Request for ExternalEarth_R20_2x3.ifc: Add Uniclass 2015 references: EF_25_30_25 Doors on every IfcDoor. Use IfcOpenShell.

First a look at what the model holds.

```python
import ifcopenshell

model = ifcopenshell.open("ExternalEarth_R20_2x3.ifc")
print(model.schema)
print("classifications:", [c.Name for c in model.by_type("IfcClassification")])
for ifc_class in ("IfcDoor", "IfcRoof", "IfcStair", "IfcWall", "IfcWindow"):
    print(ifc_class, len(model.by_type(ifc_class)))
```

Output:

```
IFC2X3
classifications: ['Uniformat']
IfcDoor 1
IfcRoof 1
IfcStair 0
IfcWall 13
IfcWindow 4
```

```python
import ifcopenshell
import ifcopenshell.api.classification

model = ifcopenshell.open("ExternalEarth_R20_2x3.ifc")

# IFC2X3 requires Source and Edition and has no link from the project to the system.
system = model.create_entity("IfcClassification", Source="NBS", Edition="2015", Name="Uniclass 2015")

codes = {
    "IfcDoor": ("EF_25_30_25", "Doors"),
}
for ifc_class, (code, name) in codes.items():
    products = model.by_type(ifc_class)
    ifcopenshell.api.classification.add_reference(
        model, products=products, classification=system, identification=code, name=name
    )
    print(code, len(products))

model.write("ExternalEarth_R20_2x3_rev.ifc")
```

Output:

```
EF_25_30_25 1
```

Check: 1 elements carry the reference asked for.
